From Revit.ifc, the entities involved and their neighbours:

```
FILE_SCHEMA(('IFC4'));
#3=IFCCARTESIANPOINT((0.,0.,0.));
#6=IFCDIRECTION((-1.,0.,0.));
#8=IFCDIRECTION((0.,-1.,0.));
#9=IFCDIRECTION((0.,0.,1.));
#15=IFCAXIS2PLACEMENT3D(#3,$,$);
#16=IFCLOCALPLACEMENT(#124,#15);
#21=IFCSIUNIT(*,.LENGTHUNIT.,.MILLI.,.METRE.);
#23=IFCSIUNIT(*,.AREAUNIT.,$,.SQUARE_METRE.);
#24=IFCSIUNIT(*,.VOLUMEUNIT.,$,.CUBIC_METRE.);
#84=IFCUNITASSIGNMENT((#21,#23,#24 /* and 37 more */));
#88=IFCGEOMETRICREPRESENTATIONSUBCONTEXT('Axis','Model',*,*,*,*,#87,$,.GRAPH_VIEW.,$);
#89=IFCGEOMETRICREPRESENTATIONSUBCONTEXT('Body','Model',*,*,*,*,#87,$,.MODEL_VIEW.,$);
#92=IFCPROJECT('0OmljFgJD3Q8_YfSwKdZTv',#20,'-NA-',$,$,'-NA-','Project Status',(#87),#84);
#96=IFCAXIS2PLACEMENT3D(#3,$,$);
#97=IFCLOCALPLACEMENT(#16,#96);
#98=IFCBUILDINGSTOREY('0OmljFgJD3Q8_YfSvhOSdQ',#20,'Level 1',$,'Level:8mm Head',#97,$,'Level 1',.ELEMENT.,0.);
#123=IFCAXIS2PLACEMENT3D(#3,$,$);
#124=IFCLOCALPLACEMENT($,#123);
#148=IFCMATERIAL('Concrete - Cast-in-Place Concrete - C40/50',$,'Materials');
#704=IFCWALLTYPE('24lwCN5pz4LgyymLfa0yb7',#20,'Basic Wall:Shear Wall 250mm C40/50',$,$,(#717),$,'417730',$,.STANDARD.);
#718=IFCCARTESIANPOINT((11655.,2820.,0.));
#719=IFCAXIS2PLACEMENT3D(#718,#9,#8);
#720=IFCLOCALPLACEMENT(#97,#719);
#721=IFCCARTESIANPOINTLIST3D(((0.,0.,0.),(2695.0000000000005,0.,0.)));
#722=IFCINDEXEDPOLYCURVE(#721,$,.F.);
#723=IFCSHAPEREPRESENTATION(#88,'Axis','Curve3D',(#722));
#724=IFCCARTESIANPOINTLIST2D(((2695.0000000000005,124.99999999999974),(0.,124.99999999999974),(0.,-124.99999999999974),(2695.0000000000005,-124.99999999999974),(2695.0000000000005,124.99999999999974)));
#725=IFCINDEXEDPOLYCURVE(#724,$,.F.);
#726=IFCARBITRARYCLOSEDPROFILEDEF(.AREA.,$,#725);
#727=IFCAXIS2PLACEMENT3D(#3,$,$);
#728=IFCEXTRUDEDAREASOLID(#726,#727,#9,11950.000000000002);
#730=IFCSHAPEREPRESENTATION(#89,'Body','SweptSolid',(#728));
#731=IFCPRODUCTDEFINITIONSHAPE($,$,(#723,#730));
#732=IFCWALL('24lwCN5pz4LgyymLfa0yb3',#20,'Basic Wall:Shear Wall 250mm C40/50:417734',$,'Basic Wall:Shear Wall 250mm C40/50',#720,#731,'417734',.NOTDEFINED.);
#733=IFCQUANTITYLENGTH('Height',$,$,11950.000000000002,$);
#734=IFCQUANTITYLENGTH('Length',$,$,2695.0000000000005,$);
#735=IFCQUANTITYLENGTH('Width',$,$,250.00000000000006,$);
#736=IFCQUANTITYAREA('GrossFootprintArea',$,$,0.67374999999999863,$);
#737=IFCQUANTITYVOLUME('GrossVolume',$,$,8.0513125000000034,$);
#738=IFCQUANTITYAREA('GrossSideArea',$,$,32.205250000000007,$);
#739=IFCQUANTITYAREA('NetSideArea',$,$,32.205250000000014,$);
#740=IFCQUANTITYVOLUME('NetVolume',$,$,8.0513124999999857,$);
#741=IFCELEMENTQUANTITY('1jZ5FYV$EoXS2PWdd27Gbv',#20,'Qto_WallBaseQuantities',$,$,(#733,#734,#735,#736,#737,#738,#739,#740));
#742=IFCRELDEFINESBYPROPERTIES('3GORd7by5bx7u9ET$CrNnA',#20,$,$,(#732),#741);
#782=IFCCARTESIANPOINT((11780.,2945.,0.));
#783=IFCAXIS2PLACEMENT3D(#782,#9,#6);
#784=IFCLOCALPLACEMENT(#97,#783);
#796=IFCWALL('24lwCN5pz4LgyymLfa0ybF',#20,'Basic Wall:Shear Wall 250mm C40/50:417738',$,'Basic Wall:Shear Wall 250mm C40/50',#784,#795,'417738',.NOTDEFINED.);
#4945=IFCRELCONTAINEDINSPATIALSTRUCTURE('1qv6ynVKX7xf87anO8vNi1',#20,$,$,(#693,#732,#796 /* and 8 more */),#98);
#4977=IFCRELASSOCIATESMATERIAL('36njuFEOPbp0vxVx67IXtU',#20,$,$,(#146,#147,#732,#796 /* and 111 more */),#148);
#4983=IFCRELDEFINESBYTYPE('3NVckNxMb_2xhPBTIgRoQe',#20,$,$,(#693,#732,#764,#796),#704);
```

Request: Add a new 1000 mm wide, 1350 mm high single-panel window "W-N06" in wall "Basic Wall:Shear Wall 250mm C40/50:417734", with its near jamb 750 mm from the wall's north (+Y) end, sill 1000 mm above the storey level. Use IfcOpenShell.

```python
import numpy as np
import ifcopenshell
import ifcopenshell.api.feature
import ifcopenshell.api.geometry
import ifcopenshell.api.pset
import ifcopenshell.api.root
import ifcopenshell.api.spatial
import ifcopenshell.geom
import ifcopenshell.util.element
import ifcopenshell.util.placement
import ifcopenshell.util.representation
import ifcopenshell.util.shape
import ifcopenshell.util.unit

model = ifcopenshell.open("Revit.ifc")
unit_scale = ifcopenshell.util.unit.calculate_unit_scale(model)
area_scale = ifcopenshell.util.unit.calculate_unit_scale(model, "AREAUNIT")
volume_scale = ifcopenshell.util.unit.calculate_unit_scale(model, "VOLUMEUNIT")
settings = ifcopenshell.geom.settings()


def volume(element):
    """Net volume in cubic metres, openings subtracted."""
    shape = ifcopenshell.geom.create_shape(settings, element)
    return ifcopenshell.util.shape.get_volume(shape.geometry)


wall = model.by_guid("24lwCN5pz4LgyymLfa0yb3")
storey = ifcopenshell.util.element.get_container(wall, ifc_class="IfcBuildingStorey")
context = ifcopenshell.util.representation.get_context(model, "Model", "Body", "MODEL_VIEW")
before = volume(wall)

width, height, from_end, sill = 1, 1.35, 0.75, 1  # metres

# The wall runs along its own X axis, and the end named is its -X end.
wall_shape = ifcopenshell.geom.create_shape(settings, wall)
x, y, z = ifcopenshell.util.shape.get_vertices(wall_shape.geometry).T
start = x.min() + from_end
face, thickness = float(y.min()), float(y.max() - y.min())
wall_matrix = ifcopenshell.util.placement.get_local_placement(wall.ObjectPlacement)
level = ifcopenshell.util.placement.get_local_placement(storey.ObjectPlacement)[2, 3]


def in_wall(x, y):
    """Placement at x, y metres in the wall's axes, at sill height."""
    matrix = wall_matrix.copy()
    matrix[:, 3] = wall_matrix @ np.array([x / unit_scale, y / unit_scale, 0.0, 1.0])
    matrix[2, 3] = level + sill / unit_scale
    return matrix


# Opening: a box that overshoots both wall faces by 50 mm.
opening = ifcopenshell.api.root.create_entity(model, ifc_class="IfcOpeningElement", predefined_type="OPENING")
box = ifcopenshell.api.geometry.add_wall_representation(
    model, context=context, length=width, height=height, thickness=thickness + 0.1
)
ifcopenshell.api.geometry.assign_representation(model, product=opening, representation=box)
ifcopenshell.api.geometry.edit_object_placement(model, product=opening, matrix=in_wall(start, face - 0.05), is_si=False)
ifcopenshell.api.feature.add_feature(model, feature=opening, element=wall)

window = ifcopenshell.api.root.create_entity(model, ifc_class="IfcWindow", name="W-N06", predefined_type="WINDOW")
window.OverallWidth, window.OverallHeight = width / unit_scale, height / unit_scale
window.PartitioningType = "SINGLE_PANEL"
body = ifcopenshell.api.geometry.add_window_representation(
    model,
    context=context,
    overall_width=window.OverallWidth,
    overall_height=window.OverallHeight,
    partition_type="SINGLE_PANEL",
)
ifcopenshell.api.geometry.assign_representation(model, product=window, representation=body)
ifcopenshell.api.spatial.assign_container(model, products=[window], relating_structure=storey)
ifcopenshell.api.feature.add_filling(model, opening=opening, element=window)

# Centre the window in the wall's thickness.
ifcopenshell.api.geometry.edit_object_placement(model, product=window, matrix=in_wall(start, face), is_si=False)
window_shape = ifcopenshell.geom.create_shape(settings, window)
depth = ifcopenshell.util.shape.get_vertices(window_shape.geometry)[:, 1]
offset = face + thickness / 2 - (depth.min() + depth.max()) / 2
ifcopenshell.api.geometry.edit_object_placement(model, product=window, matrix=in_wall(start, offset), is_si=False)

after = volume(wall)

# Update the wall's stored quantities.
qto = model.by_id(ifcopenshell.util.element.get_pset(wall, "Qto_WallBaseQuantities", should_inherit=False)["id"])
ifcopenshell.api.pset.edit_qto(model, qto=qto, properties={
    "NetSideArea": after / thickness / area_scale,
    "NetVolume": after / volume_scale,
})

print(f"wall volume {before:.3f} -> {after:.3f} m3")

model.write("Revit_updated.ifc")
```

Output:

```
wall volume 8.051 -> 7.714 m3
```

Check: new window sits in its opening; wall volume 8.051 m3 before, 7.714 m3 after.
